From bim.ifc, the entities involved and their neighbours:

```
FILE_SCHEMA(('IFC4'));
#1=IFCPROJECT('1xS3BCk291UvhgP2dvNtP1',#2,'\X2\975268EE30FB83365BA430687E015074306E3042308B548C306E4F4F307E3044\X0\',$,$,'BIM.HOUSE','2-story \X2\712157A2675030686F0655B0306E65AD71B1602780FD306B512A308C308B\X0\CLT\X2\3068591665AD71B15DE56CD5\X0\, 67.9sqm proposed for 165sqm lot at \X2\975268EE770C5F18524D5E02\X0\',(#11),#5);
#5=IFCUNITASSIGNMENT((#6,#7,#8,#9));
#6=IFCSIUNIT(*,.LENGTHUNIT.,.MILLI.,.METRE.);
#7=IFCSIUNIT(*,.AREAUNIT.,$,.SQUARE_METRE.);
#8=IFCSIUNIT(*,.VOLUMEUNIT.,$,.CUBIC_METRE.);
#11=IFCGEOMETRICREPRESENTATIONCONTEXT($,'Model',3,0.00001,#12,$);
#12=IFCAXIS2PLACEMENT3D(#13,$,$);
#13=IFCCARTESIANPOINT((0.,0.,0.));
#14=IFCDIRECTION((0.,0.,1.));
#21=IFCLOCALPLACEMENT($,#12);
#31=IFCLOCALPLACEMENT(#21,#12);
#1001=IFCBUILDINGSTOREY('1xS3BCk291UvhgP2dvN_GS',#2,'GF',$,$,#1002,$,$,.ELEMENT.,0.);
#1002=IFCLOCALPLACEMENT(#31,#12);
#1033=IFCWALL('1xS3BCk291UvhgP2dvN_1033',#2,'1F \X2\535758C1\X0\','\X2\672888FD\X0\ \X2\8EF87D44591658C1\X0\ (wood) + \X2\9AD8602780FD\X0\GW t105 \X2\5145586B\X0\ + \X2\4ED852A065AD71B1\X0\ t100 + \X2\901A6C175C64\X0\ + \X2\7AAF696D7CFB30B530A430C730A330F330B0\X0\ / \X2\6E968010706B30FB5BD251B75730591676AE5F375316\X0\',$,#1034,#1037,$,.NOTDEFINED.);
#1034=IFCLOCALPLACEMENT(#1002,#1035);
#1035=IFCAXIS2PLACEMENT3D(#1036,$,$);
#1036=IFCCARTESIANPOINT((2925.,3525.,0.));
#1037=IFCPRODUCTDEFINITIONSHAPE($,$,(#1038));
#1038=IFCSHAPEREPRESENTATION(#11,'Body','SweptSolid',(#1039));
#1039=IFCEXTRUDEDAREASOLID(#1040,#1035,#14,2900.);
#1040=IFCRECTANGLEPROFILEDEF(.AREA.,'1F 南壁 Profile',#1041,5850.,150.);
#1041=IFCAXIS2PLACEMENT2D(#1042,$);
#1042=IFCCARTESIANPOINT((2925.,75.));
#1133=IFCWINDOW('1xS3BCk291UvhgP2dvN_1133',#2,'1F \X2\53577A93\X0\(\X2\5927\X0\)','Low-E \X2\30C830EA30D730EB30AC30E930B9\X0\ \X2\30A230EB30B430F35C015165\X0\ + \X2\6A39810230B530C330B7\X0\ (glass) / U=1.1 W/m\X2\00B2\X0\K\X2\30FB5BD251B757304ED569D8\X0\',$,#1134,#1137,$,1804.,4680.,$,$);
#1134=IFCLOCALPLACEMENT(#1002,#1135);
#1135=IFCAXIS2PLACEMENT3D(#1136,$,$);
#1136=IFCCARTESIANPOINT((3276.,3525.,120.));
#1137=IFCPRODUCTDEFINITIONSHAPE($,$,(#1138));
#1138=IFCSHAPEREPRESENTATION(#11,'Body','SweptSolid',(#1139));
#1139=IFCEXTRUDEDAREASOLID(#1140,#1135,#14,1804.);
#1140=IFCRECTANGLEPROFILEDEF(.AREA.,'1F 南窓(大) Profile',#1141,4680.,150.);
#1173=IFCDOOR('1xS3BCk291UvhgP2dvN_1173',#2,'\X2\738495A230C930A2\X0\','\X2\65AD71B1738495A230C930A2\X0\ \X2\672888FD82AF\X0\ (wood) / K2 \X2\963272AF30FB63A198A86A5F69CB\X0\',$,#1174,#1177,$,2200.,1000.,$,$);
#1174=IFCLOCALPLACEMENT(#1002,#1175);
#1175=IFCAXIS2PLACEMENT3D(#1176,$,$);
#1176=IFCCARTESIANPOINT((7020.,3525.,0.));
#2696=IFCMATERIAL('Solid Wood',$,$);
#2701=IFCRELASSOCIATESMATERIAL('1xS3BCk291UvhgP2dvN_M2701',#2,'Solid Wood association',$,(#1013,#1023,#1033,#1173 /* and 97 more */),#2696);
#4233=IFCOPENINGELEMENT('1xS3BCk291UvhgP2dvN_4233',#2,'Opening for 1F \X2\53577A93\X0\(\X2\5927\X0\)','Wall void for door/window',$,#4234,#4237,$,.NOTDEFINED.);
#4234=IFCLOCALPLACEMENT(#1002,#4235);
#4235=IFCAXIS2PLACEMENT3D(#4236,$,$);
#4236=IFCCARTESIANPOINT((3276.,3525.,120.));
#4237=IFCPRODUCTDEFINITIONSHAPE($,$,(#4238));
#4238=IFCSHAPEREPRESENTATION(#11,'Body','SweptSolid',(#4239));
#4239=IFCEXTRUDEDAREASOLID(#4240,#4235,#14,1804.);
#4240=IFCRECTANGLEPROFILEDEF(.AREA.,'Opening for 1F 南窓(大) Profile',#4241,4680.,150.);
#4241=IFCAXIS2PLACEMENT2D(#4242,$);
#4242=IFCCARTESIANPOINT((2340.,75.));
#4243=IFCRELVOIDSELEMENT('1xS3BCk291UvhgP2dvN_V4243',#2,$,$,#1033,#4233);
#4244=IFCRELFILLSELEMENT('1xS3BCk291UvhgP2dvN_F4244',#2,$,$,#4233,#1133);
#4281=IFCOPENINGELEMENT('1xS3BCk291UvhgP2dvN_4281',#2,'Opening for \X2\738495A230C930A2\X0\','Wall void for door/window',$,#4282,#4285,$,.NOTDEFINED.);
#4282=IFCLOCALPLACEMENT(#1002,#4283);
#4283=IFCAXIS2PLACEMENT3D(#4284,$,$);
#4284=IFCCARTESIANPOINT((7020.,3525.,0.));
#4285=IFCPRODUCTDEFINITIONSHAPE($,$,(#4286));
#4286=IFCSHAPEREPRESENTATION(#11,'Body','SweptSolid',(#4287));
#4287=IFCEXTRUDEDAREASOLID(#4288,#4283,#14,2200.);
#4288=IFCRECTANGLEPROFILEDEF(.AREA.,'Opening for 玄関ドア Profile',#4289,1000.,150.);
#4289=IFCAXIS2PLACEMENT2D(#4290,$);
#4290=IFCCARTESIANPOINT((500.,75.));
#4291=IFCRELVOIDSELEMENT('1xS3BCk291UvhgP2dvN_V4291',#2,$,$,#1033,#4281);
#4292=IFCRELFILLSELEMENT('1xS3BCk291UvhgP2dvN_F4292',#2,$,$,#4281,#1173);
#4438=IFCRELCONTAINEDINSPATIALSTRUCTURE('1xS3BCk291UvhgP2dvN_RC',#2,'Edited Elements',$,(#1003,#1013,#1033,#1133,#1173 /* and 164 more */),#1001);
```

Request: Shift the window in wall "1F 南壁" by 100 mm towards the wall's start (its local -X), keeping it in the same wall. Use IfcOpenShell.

```python
import ifcopenshell
import ifcopenshell.api.geometry
import ifcopenshell.util.placement

model = ifcopenshell.open("bim.ifc")

window = model.by_guid("1xS3BCk291UvhgP2dvN_1133")
opening = window.FillsVoids[0].RelatingOpeningElement
wall = opening.VoidsElements[0].RelatingBuildingElement

wall_matrix = ifcopenshell.util.placement.get_local_placement(wall.ObjectPlacement)
shift = wall_matrix[:3, 0] * -100.0
before = ifcopenshell.util.placement.get_local_placement(window.ObjectPlacement)[:3, 3].copy()

# The window is not placed relative to its opening, so move both.
for product in (opening, window):
    matrix = ifcopenshell.util.placement.get_local_placement(product.ObjectPlacement)
    matrix[:3, 3] += shift
    ifcopenshell.api.geometry.edit_object_placement(model, product=product, matrix=matrix, is_si=False)

after = ifcopenshell.util.placement.get_local_placement(window.ObjectPlacement)[:3, 3]
print("window moved by", (after - before).round(3) + 0.0)

model.write("bim_rev.ifc")
```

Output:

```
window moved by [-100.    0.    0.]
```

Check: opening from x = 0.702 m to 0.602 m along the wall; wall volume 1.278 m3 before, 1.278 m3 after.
